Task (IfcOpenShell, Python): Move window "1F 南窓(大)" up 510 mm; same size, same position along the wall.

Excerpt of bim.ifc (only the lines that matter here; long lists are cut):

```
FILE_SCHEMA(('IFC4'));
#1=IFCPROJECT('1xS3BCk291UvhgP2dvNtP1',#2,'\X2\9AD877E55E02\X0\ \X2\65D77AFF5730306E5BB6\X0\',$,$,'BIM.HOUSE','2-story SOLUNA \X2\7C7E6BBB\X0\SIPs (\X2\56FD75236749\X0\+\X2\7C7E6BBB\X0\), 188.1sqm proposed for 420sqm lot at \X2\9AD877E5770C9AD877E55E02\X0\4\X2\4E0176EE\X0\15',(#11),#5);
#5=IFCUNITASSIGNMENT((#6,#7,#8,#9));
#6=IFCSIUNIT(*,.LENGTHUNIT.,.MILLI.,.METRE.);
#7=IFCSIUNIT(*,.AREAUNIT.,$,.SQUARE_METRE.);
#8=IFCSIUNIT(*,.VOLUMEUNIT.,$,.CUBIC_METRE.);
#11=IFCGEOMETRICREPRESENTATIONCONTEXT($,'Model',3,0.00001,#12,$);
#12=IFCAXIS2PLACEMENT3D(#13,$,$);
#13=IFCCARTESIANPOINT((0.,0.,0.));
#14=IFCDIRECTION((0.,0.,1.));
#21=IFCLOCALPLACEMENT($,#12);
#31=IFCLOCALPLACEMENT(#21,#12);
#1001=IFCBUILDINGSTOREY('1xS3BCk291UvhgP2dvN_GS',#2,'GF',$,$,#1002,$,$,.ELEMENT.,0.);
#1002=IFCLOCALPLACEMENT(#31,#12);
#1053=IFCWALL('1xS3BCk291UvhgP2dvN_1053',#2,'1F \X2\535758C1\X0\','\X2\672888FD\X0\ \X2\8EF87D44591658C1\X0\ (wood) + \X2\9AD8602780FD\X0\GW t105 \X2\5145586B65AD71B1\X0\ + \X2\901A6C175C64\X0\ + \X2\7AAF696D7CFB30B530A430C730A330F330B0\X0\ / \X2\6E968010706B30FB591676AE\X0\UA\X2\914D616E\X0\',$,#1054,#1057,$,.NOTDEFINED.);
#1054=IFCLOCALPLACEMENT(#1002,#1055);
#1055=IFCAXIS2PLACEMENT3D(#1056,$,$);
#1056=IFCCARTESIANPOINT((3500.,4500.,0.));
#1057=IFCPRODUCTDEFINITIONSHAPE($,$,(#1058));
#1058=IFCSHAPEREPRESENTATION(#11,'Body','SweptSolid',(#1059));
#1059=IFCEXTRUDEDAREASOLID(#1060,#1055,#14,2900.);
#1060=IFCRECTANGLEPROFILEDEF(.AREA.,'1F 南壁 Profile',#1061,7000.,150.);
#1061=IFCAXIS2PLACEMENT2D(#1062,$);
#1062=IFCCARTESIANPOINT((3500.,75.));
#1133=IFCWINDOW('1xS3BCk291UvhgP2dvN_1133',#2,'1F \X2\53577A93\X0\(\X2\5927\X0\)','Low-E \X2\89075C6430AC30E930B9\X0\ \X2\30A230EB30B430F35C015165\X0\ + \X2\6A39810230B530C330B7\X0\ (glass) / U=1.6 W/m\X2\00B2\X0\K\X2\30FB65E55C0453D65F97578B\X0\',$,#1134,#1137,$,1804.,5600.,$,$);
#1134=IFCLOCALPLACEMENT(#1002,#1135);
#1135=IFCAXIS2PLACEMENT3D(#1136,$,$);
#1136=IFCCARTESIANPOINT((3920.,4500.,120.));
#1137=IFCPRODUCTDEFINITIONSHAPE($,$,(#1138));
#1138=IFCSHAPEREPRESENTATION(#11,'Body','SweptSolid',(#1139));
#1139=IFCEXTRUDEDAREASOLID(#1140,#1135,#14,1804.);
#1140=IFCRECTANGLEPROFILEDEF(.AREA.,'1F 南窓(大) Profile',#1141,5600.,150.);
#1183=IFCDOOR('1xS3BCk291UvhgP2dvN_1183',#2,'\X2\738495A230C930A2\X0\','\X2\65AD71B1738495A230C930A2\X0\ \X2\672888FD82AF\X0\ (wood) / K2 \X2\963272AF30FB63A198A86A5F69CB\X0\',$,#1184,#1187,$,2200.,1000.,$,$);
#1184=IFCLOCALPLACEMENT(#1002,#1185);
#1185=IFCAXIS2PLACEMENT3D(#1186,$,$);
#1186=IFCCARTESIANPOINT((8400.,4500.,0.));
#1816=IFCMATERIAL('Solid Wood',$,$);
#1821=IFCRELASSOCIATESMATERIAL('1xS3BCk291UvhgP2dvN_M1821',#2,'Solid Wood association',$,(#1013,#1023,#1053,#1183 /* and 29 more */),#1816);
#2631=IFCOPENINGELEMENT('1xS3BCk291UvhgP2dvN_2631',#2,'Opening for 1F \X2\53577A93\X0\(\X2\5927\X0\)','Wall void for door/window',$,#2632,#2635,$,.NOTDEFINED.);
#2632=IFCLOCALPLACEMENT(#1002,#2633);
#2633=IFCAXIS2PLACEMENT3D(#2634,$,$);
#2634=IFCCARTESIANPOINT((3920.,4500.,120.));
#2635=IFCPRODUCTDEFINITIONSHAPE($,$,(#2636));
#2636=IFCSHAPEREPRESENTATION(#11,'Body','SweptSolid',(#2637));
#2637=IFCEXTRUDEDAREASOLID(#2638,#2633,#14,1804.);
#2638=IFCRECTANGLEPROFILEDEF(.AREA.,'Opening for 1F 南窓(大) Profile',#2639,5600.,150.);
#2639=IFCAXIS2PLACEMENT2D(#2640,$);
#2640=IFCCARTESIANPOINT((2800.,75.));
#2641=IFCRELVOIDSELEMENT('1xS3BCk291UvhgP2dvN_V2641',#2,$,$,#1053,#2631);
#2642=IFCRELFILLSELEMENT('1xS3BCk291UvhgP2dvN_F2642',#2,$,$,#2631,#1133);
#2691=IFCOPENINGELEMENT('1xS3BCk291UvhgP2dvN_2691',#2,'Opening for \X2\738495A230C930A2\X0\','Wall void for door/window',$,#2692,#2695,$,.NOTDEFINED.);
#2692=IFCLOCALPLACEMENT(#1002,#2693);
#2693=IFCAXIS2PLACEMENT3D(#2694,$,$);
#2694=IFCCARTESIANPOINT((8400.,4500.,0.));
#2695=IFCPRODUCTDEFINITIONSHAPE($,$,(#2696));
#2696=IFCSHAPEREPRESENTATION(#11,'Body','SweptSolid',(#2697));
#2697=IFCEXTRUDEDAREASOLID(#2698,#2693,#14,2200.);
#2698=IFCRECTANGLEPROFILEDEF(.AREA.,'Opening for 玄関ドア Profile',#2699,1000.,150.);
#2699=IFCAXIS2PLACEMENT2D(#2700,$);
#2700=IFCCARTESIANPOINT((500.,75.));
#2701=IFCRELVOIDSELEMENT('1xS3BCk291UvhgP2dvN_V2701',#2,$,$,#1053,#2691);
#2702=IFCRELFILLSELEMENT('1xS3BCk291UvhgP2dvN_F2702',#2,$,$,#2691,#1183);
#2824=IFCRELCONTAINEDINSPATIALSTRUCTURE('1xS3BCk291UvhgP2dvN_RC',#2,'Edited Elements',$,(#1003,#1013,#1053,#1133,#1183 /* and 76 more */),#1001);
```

```python
import numpy as np
import ifcopenshell
import ifcopenshell.api.geometry
import ifcopenshell.util.placement
import ifcopenshell.util.unit

model = ifcopenshell.open("bim.ifc")
unit_scale = ifcopenshell.util.unit.calculate_unit_scale(model)

window = model.by_guid("1xS3BCk291UvhgP2dvN_1133")
opening = window.FillsVoids[0].RelatingOpeningElement
dz = 0.51 / unit_scale

shift = np.array([0.0, 0.0, dz])
# The window is not placed relative to its opening, so move both.
for product in (opening, window):
    matrix = ifcopenshell.util.placement.get_local_placement(product.ObjectPlacement)
    matrix[:3, 3] += shift
    ifcopenshell.api.geometry.edit_object_placement(model, product=product, matrix=matrix, is_si=False)

print(f"moved by {dz * unit_scale:+.3f} m")

model.write("bim-out.ifc")
```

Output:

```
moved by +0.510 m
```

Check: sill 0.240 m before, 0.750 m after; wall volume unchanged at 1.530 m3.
